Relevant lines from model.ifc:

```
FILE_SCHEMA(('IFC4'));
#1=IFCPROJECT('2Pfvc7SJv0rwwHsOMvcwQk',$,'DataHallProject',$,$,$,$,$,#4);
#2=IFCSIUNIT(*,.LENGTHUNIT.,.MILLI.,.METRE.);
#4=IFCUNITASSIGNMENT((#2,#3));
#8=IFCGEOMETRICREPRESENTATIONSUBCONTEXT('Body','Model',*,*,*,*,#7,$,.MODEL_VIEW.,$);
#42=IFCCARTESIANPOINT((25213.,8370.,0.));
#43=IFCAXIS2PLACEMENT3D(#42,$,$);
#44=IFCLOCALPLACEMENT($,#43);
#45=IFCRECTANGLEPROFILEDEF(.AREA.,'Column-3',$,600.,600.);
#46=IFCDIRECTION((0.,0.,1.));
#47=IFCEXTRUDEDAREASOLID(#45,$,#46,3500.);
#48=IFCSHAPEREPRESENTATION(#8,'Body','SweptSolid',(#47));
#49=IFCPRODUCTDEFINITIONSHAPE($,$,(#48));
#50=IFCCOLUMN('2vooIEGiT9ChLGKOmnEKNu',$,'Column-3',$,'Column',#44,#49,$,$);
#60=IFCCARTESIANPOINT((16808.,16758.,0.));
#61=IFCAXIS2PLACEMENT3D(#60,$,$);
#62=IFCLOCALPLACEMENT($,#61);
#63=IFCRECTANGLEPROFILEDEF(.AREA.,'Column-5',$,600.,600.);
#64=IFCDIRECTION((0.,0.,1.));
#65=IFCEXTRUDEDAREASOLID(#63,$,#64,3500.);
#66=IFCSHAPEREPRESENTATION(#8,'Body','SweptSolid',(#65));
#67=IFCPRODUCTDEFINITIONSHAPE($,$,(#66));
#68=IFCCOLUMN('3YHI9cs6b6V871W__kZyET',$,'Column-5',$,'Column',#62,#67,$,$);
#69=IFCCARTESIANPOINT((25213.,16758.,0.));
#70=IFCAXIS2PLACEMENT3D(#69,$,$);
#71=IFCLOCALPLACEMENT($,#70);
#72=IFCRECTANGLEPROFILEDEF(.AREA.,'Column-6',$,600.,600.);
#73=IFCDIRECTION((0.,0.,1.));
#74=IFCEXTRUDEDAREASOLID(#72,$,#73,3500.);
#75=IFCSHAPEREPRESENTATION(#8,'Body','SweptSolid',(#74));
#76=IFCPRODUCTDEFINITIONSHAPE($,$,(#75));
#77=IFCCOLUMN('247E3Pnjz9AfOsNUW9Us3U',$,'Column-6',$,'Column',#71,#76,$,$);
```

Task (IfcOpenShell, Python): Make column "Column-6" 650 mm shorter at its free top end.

```python
import ifcopenshell
import ifcopenshell.util.representation
import ifcopenshell.util.unit

model = ifcopenshell.open("model.ifc")
unit_scale = ifcopenshell.util.unit.calculate_unit_scale(model)

member = model.by_guid("247E3Pnjz9AfOsNUW9Us3U")
change = -0.65 / unit_scale

# The extrusion runs towards the end named, so only its depth changes.
body = ifcopenshell.util.representation.get_representation(member, "Model", "Body")
solid = body.Items[0]
old_length = solid.Depth
solid.Depth += change

print(f"length {old_length:g} -> {solid.Depth:g}")

model.write("model_updated.ifc")
```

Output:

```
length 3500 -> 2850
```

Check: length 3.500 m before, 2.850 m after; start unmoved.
